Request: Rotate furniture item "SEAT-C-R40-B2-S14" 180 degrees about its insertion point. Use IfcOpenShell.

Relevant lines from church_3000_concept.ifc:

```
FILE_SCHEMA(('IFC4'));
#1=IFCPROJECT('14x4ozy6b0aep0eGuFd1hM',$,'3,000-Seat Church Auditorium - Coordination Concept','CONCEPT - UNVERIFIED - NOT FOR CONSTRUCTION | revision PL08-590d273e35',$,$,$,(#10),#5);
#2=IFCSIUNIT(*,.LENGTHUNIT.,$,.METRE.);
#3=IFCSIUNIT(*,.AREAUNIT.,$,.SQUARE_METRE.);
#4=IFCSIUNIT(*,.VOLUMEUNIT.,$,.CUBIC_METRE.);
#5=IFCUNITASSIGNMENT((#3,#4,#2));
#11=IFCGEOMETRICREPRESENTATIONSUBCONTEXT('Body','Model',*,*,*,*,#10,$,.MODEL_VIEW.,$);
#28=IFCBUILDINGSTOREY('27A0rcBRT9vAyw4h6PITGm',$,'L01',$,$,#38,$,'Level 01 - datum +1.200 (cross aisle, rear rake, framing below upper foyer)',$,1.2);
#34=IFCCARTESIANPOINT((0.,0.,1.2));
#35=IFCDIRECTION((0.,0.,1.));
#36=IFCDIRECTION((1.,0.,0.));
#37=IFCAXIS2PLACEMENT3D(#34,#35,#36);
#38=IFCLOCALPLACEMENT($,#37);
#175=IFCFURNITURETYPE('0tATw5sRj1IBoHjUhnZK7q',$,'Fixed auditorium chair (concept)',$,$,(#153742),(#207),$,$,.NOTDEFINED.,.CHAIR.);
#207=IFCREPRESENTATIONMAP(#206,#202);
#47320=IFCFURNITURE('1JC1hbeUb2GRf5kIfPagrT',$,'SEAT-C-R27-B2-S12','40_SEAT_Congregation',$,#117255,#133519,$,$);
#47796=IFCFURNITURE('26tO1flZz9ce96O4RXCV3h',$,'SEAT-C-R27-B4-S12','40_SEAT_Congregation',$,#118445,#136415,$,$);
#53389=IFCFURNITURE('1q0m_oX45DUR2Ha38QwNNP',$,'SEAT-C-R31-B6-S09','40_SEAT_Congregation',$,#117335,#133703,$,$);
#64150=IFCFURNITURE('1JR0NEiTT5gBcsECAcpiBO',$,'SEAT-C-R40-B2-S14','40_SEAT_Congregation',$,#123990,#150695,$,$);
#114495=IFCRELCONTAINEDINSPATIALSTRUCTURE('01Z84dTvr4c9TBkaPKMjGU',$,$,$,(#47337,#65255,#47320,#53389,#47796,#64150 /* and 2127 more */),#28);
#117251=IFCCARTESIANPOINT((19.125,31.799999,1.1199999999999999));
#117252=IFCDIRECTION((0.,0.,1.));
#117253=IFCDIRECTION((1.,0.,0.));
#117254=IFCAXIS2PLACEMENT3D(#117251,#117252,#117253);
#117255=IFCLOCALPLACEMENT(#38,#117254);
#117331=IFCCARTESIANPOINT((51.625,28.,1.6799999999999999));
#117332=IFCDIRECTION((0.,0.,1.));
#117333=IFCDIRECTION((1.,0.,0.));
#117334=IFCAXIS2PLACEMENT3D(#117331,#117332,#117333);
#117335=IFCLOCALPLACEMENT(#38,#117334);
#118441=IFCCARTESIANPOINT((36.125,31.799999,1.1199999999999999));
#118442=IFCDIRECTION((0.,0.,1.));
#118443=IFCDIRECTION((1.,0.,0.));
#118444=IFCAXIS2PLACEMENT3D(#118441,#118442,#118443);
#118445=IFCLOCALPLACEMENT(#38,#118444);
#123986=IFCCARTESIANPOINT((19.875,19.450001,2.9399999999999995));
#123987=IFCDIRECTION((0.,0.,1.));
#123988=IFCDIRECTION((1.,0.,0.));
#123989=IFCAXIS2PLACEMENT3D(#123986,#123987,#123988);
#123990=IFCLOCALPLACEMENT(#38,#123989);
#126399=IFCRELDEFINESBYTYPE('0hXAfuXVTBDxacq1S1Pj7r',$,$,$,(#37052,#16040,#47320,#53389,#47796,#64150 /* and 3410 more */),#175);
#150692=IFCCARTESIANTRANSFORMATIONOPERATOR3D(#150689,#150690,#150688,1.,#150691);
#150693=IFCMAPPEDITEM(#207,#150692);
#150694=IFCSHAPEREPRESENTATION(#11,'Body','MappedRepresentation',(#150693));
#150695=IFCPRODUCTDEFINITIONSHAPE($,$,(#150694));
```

```python
import ifcopenshell
import ifcopenshell.api.geometry
import ifcopenshell.util.placement

model = ifcopenshell.open("church_3000_concept.ifc")

item = model.by_guid("1JR0NEiTT5gBcsECAcpiBO")
matrix = ifcopenshell.util.placement.get_local_placement(item.ObjectPlacement)
matrix = matrix @ ifcopenshell.util.placement.rotation(180, "Z")
ifcopenshell.api.geometry.edit_object_placement(model, product=item, matrix=matrix, is_si=False)

print(ifcopenshell.util.placement.get_local_placement(item.ObjectPlacement).round(3) + 0.0)

model.write("church_3000_concept_v2.ifc")
```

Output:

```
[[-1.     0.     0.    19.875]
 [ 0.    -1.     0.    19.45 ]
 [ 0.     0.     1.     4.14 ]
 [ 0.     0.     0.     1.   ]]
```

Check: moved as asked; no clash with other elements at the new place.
